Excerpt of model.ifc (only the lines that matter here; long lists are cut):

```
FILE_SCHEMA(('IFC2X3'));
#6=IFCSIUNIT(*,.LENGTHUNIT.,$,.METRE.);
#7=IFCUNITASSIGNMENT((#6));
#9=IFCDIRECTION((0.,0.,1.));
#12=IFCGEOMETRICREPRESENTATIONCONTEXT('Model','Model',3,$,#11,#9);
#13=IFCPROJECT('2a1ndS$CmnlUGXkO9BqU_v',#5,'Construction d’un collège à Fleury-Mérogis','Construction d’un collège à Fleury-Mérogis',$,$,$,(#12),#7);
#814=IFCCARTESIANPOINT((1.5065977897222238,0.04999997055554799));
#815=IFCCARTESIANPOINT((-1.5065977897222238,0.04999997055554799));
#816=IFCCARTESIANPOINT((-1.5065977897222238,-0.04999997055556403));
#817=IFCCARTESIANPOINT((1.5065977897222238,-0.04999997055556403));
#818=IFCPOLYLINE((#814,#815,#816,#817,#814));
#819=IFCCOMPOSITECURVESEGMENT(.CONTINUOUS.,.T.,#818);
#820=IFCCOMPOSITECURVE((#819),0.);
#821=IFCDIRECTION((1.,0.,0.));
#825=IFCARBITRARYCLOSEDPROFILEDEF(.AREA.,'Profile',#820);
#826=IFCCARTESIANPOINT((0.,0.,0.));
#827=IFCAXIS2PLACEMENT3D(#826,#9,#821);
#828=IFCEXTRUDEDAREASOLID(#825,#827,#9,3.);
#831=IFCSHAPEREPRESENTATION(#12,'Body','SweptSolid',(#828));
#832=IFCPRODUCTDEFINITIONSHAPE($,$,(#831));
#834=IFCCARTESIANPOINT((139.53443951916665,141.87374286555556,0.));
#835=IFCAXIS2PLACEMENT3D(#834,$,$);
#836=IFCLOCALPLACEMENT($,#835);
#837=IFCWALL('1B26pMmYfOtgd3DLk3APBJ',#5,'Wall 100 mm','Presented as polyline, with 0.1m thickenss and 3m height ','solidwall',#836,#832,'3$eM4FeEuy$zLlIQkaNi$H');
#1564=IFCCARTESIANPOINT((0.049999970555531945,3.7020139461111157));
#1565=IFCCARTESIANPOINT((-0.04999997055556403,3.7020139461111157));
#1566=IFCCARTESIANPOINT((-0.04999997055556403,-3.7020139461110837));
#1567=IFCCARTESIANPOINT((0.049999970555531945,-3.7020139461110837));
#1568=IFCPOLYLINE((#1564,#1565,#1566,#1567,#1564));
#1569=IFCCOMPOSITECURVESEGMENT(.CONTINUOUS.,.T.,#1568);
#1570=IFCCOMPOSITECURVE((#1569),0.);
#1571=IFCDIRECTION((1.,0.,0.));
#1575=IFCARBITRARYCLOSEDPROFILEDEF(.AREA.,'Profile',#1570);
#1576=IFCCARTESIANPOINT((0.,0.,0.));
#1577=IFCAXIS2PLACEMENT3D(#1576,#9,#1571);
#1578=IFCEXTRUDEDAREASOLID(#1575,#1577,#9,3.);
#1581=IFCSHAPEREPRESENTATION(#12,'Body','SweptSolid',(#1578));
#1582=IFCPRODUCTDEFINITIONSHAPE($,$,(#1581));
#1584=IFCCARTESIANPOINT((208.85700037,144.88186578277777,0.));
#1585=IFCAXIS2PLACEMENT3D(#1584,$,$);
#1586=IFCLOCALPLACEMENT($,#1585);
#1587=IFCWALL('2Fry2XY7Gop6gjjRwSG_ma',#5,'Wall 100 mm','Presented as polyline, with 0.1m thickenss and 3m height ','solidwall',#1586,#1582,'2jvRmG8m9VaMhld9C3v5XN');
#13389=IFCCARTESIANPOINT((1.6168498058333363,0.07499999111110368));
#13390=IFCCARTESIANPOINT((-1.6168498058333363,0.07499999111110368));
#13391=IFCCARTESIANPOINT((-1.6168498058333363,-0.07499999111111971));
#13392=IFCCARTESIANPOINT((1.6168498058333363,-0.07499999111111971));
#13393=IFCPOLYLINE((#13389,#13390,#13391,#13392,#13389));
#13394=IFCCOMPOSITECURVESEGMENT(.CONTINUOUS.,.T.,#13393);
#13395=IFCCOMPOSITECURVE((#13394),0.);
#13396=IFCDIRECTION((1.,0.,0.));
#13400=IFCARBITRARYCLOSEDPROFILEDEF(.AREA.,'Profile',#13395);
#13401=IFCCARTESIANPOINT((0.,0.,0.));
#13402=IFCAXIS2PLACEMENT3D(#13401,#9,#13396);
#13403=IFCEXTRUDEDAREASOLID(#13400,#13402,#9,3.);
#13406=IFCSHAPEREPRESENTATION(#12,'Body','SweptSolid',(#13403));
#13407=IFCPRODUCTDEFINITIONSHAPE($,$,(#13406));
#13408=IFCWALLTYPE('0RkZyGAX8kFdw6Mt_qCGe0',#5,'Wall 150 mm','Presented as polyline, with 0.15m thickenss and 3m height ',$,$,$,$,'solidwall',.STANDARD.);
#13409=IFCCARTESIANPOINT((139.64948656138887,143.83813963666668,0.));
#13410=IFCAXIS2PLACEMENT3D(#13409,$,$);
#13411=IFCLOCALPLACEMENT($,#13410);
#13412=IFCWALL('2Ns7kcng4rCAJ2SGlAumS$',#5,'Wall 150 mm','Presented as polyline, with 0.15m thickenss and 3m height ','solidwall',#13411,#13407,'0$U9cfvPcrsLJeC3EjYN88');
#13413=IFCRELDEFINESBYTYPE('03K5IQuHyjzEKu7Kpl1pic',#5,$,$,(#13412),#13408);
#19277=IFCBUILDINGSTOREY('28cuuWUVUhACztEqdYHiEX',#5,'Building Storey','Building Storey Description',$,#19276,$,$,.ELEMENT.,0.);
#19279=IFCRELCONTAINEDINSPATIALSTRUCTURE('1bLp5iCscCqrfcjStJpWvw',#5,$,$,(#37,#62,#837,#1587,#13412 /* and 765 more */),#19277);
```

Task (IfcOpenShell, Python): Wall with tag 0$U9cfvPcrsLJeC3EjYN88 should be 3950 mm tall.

```python
import ifcopenshell
import ifcopenshell.geom
import ifcopenshell.util.shape

model = ifcopenshell.open("model.ifc")
settings = ifcopenshell.geom.settings()


def volume(element):
    """Net volume in cubic metres, openings subtracted."""
    shape = ifcopenshell.geom.create_shape(settings, element)
    return ifcopenshell.util.shape.get_volume(shape.geometry)


wall = model.by_guid("2Ns7kcng4rCAJ2SGlAumS$")
before = volume(wall)

body = next(r for r in wall.Representation.Representations if r.RepresentationIdentifier == "Body")
solid = body.Items[0]
old_height = solid.Depth
solid.Depth = 3.95
after = volume(wall)

print(f"height {old_height:g} -> {solid.Depth:g}, volume {before:.3f} -> {after:.3f} m3")

model.write("model_updated.ifc")
```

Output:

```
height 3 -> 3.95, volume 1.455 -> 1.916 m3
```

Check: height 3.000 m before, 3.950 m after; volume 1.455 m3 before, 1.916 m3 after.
